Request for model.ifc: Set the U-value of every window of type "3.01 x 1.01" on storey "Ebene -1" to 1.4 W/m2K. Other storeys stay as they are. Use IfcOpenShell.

First a look at what the model holds.

```python
import ifcopenshell
import ifcopenshell.util.element

model = ifcopenshell.open("model.ifc")
print(model.schema)
storey = next(s for s in model.by_type("IfcBuildingStorey") if s.Name == "Ebene -1")
windows = [e for e in ifcopenshell.util.element.get_decomposition(storey) if e.is_a("IfcWindow")]
seen = {}
for e in windows:
    element_type = ifcopenshell.util.element.get_type(e)
    key = (element_type.Name if element_type != e and element_type else None, ifcopenshell.util.element.get_pset(e, "Pset_WindowCommon", "ThermalTransmittance"))
    seen[key] = seen.get(key, 0) + 1
for (name, value), count in sorted(seen.items(), key=str):
    print(count, "x", name, "|", value)
```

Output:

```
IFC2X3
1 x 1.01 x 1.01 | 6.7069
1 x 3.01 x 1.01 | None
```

```python
import ifcopenshell
import ifcopenshell.api.pset
import ifcopenshell.util.element

model = ifcopenshell.open("model.ifc")

storey = next(s for s in model.by_type("IfcBuildingStorey") if s.Name == "Ebene -1")
windows = [e for e in ifcopenshell.util.element.get_decomposition(storey) if e.is_a("IfcWindow")]

count = 0
for e in windows:
    element_type = ifcopenshell.util.element.get_type(e)
    if element_type in (None, e) or element_type.Name != "3.01 x 1.01":
        continue
    # add_pset returns the element's existing set when there is one.
    pset = ifcopenshell.api.pset.add_pset(model, product=e, name="Pset_WindowCommon")
    ifcopenshell.api.pset.edit_pset(model, pset=pset, properties={"ThermalTransmittance": 1.4})
    count += 1

print(count, "windows updated")

model.write("model_v2.ifc")
```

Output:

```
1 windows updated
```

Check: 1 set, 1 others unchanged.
